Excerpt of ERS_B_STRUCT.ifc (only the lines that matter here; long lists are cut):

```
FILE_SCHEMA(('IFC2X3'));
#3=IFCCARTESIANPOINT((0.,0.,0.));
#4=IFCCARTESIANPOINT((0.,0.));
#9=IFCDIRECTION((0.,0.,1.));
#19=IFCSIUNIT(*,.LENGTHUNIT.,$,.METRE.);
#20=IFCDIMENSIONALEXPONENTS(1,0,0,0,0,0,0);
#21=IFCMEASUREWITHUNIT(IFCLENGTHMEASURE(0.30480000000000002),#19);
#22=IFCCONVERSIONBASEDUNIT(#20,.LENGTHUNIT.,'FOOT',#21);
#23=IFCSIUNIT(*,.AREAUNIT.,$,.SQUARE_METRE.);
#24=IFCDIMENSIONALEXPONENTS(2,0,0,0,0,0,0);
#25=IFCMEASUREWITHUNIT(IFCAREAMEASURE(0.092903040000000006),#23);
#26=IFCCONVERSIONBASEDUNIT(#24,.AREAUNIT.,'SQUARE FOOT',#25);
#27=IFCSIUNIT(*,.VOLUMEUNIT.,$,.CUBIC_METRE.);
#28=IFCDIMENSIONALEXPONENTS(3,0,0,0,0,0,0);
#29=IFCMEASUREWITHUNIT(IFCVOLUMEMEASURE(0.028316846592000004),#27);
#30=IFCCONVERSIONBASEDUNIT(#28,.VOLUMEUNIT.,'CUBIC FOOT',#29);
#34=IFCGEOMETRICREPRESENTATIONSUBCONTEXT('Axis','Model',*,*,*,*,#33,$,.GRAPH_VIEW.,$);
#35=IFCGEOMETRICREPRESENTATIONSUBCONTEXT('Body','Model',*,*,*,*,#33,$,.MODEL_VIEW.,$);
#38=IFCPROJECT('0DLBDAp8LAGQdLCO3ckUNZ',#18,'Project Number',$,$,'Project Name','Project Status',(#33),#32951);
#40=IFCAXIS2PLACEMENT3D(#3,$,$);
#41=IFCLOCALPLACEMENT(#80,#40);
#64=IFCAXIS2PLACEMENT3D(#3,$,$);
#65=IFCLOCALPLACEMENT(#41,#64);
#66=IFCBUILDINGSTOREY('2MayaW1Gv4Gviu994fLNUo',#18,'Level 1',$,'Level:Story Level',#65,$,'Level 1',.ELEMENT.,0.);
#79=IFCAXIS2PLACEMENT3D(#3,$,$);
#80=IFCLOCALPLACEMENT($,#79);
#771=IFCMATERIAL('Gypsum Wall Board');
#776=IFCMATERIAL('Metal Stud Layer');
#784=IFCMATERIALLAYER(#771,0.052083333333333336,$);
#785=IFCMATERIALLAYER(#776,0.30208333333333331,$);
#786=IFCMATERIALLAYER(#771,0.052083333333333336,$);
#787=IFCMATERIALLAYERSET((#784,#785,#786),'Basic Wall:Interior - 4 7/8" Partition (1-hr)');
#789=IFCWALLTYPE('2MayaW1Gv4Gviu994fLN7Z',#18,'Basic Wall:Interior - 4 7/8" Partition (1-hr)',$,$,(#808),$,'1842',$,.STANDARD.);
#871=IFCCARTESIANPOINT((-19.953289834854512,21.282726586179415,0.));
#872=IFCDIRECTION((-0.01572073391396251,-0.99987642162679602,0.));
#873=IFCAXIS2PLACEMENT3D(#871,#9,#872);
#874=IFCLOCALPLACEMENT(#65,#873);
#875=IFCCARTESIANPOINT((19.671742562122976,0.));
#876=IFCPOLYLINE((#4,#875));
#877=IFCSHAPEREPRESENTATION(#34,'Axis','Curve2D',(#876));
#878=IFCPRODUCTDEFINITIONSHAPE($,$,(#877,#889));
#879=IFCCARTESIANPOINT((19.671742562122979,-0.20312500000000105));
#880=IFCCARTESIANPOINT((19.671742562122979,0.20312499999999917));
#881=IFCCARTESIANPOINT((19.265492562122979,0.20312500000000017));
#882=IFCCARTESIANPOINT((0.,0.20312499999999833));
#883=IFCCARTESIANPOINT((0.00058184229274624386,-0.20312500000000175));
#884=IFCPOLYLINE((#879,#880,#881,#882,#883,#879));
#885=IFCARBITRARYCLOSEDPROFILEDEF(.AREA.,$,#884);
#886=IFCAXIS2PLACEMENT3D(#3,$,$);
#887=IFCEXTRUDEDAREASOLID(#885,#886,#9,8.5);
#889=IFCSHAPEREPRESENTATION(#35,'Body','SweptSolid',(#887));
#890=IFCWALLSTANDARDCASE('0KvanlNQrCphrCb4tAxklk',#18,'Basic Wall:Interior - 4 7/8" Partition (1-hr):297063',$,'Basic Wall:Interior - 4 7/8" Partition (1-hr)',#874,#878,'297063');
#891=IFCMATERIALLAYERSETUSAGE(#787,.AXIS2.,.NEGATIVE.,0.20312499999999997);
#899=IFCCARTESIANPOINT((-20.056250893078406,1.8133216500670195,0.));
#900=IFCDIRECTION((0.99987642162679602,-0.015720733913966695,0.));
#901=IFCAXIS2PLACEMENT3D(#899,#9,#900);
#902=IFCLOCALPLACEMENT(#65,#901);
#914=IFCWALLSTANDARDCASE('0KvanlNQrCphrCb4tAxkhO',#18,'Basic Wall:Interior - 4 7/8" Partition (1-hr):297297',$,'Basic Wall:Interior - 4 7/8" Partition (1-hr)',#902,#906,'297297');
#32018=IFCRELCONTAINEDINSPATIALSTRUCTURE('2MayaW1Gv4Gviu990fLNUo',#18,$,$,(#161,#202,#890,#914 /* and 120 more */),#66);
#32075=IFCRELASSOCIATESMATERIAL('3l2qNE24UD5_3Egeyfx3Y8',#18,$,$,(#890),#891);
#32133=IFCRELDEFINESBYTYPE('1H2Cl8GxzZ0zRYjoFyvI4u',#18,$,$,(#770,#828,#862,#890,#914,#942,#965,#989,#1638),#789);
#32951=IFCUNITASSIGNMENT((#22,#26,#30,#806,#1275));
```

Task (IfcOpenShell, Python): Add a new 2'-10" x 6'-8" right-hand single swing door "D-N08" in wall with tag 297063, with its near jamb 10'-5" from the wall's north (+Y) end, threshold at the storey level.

```python
import numpy as np
import ifcopenshell
import ifcopenshell.api.feature
import ifcopenshell.api.geometry
import ifcopenshell.api.root
import ifcopenshell.api.spatial
import ifcopenshell.api.type
import ifcopenshell.geom
import ifcopenshell.util.element
import ifcopenshell.util.placement
import ifcopenshell.util.representation
import ifcopenshell.util.shape
import ifcopenshell.util.unit

model = ifcopenshell.open("ERS_B_STRUCT.ifc")
unit_scale = ifcopenshell.util.unit.calculate_unit_scale(model)
settings = ifcopenshell.geom.settings()


def volume(element):
    """Net volume in cubic metres, openings subtracted."""
    shape = ifcopenshell.geom.create_shape(settings, element)
    return ifcopenshell.util.shape.get_volume(shape.geometry)


wall = model.by_guid("0KvanlNQrCphrCb4tAxklk")
storey = ifcopenshell.util.element.get_container(wall, ifc_class="IfcBuildingStorey")
context = ifcopenshell.util.representation.get_context(model, "Model", "Body", "MODEL_VIEW")
before = volume(wall)

width, height, from_end, sill = 0.8636, 2.032, 3.175, 0.0  # metres

# The wall runs along its own X axis, and the end named is its -X end.
wall_shape = ifcopenshell.geom.create_shape(settings, wall)
x, y, z = ifcopenshell.util.shape.get_vertices(wall_shape.geometry).T
start = x.min() + from_end
face, thickness = float(y.min()), float(y.max() - y.min())
wall_matrix = ifcopenshell.util.placement.get_local_placement(wall.ObjectPlacement)
level = ifcopenshell.util.placement.get_local_placement(storey.ObjectPlacement)[2, 3]


def in_wall(x, y):
    """Placement at x, y metres in the wall's axes, at sill height."""
    matrix = wall_matrix.copy()
    matrix[:, 3] = wall_matrix @ np.array([x / unit_scale, y / unit_scale, 0.0, 1.0])
    matrix[2, 3] = level + sill / unit_scale
    return matrix


# Opening: a box that overshoots both wall faces by 50 mm.
opening = ifcopenshell.api.root.create_entity(model, ifc_class="IfcOpeningElement")
box = ifcopenshell.api.geometry.add_wall_representation(
    model, context=context, length=width, height=height, thickness=thickness + 0.1
)
ifcopenshell.api.geometry.assign_representation(model, product=opening, representation=box)
ifcopenshell.api.geometry.edit_object_placement(model, product=opening, matrix=in_wall(start, face - 0.05), is_si=False)
ifcopenshell.api.feature.add_feature(model, feature=opening, element=wall)

door = ifcopenshell.api.root.create_entity(model, ifc_class="IfcDoor", name="D-N08")
door.OverallWidth, door.OverallHeight = width / unit_scale, height / unit_scale
body = ifcopenshell.api.geometry.add_door_representation(
    model,
    context=context,
    overall_width=door.OverallWidth,
    overall_height=door.OverallHeight,
    operation_type="SINGLE_SWING_RIGHT",
    lining_properties={"LiningDepth": thickness / unit_scale, "ThresholdDepth": thickness / unit_scale},
)
ifcopenshell.api.geometry.assign_representation(model, product=door, representation=body)
ifcopenshell.api.spatial.assign_container(model, products=[door], relating_structure=storey)
fills = ifcopenshell.api.feature.add_filling(model, opening=opening, element=door)
fills.OwnerHistory = door.OwnerHistory  # required in IFC2X3

# IFC2X3 keeps the operation on the door style.
style = ifcopenshell.api.root.create_entity(model, ifc_class="IfcDoorStyle", name="D-N08")
style.OperationType, style.ConstructionType = "SINGLE_SWING_RIGHT", "NOTDEFINED"
style.ParameterTakesPrecedence = style.Sizeable = False
ifcopenshell.api.type.assign_type(model, related_objects=[door], relating_type=style)

# The lining spans the wall, so the door starts at the wall face.
ifcopenshell.api.geometry.edit_object_placement(model, product=door, matrix=in_wall(start, face), is_si=False)

after = volume(wall)

print(f"wall volume {before:.3f} -> {after:.3f} m3")

model.write("ERS_B_STRUCT_v2.ifc")
```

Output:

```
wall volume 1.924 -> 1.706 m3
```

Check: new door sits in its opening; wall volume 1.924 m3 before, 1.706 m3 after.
